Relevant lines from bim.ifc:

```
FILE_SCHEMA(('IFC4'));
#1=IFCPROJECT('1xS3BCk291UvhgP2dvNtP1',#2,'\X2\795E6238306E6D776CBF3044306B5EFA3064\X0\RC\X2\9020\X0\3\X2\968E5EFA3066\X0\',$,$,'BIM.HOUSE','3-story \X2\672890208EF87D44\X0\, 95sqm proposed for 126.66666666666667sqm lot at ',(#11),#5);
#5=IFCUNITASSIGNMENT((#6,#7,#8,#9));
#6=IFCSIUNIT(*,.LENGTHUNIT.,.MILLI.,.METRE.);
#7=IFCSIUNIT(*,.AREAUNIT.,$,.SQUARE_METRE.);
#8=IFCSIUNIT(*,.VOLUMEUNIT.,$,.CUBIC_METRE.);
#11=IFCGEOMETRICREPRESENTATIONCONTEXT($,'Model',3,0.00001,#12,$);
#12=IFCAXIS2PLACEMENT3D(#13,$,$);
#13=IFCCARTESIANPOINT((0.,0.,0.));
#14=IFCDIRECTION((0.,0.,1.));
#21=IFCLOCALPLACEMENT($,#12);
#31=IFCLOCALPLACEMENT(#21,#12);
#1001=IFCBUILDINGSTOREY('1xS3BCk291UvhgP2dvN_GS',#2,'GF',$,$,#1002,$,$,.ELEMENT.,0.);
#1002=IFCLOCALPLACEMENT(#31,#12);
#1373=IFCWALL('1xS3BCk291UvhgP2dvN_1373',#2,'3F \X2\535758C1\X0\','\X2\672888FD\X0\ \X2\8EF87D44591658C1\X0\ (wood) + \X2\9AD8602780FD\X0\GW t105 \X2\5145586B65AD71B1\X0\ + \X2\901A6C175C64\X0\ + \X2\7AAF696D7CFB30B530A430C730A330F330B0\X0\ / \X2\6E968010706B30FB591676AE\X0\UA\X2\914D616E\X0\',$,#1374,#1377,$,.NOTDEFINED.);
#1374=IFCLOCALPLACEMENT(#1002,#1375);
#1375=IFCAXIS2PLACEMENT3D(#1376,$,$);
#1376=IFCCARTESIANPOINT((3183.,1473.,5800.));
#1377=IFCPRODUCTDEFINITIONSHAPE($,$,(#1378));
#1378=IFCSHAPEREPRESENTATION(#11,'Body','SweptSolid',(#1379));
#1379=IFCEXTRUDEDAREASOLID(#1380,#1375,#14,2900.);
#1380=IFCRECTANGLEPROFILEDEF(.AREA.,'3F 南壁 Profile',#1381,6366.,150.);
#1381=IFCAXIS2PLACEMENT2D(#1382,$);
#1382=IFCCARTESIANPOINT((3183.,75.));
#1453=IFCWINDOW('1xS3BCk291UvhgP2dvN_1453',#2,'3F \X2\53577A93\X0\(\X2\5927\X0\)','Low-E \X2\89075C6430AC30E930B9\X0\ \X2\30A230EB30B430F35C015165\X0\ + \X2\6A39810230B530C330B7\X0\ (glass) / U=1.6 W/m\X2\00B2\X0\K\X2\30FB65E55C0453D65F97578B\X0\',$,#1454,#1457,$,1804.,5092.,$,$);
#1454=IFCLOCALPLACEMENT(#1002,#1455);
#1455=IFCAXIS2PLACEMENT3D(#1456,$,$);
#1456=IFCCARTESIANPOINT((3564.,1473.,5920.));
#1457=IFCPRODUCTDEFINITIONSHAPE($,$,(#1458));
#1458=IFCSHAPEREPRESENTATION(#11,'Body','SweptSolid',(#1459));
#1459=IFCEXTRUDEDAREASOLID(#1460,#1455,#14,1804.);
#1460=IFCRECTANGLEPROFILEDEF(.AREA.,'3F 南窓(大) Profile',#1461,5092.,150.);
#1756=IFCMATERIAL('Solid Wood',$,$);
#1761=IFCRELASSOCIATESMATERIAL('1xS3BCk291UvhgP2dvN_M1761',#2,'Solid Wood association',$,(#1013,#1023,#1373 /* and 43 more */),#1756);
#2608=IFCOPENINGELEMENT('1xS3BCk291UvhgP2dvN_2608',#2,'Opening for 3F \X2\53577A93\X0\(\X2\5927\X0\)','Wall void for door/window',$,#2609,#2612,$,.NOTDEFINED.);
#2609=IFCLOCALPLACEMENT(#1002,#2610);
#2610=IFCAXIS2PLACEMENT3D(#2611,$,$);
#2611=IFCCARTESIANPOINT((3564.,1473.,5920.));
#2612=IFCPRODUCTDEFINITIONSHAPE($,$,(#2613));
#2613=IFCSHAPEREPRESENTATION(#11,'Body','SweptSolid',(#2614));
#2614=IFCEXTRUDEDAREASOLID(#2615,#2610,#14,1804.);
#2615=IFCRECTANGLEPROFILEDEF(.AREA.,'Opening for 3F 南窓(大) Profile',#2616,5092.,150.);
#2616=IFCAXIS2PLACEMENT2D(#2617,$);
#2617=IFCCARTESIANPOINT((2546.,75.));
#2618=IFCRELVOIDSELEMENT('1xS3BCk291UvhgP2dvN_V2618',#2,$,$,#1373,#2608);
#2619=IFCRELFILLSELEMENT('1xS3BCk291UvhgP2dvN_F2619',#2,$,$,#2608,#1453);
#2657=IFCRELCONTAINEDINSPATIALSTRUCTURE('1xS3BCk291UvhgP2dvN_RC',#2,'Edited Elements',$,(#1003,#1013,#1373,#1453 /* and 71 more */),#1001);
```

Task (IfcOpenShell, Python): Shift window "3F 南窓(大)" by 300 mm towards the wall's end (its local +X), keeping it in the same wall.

```python
import ifcopenshell
import ifcopenshell.api.geometry
import ifcopenshell.util.placement
import ifcopenshell.util.unit

model = ifcopenshell.open("bim.ifc")
unit_scale = ifcopenshell.util.unit.calculate_unit_scale(model)

window = model.by_id(1453)
opening = window.FillsVoids[0].RelatingOpeningElement
wall = opening.VoidsElements[0].RelatingBuildingElement

wall_matrix = ifcopenshell.util.placement.get_local_placement(wall.ObjectPlacement)
shift = wall_matrix[:3, 0] * 0.3 / unit_scale
before = ifcopenshell.util.placement.get_local_placement(window.ObjectPlacement)[:3, 3].copy()

# The window is not placed relative to its opening, so move both.
for product in (opening, window):
    matrix = ifcopenshell.util.placement.get_local_placement(product.ObjectPlacement)
    matrix[:3, 3] += shift
    ifcopenshell.api.geometry.edit_object_placement(model, product=product, matrix=matrix, is_si=False)

after = ifcopenshell.util.placement.get_local_placement(window.ObjectPlacement)[:3, 3]
print("window moved by", (after - before).round(3) + 0.0)

model.write("bim_updated.ifc")
```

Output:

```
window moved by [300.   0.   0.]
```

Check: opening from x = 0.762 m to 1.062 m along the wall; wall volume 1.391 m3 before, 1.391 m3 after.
